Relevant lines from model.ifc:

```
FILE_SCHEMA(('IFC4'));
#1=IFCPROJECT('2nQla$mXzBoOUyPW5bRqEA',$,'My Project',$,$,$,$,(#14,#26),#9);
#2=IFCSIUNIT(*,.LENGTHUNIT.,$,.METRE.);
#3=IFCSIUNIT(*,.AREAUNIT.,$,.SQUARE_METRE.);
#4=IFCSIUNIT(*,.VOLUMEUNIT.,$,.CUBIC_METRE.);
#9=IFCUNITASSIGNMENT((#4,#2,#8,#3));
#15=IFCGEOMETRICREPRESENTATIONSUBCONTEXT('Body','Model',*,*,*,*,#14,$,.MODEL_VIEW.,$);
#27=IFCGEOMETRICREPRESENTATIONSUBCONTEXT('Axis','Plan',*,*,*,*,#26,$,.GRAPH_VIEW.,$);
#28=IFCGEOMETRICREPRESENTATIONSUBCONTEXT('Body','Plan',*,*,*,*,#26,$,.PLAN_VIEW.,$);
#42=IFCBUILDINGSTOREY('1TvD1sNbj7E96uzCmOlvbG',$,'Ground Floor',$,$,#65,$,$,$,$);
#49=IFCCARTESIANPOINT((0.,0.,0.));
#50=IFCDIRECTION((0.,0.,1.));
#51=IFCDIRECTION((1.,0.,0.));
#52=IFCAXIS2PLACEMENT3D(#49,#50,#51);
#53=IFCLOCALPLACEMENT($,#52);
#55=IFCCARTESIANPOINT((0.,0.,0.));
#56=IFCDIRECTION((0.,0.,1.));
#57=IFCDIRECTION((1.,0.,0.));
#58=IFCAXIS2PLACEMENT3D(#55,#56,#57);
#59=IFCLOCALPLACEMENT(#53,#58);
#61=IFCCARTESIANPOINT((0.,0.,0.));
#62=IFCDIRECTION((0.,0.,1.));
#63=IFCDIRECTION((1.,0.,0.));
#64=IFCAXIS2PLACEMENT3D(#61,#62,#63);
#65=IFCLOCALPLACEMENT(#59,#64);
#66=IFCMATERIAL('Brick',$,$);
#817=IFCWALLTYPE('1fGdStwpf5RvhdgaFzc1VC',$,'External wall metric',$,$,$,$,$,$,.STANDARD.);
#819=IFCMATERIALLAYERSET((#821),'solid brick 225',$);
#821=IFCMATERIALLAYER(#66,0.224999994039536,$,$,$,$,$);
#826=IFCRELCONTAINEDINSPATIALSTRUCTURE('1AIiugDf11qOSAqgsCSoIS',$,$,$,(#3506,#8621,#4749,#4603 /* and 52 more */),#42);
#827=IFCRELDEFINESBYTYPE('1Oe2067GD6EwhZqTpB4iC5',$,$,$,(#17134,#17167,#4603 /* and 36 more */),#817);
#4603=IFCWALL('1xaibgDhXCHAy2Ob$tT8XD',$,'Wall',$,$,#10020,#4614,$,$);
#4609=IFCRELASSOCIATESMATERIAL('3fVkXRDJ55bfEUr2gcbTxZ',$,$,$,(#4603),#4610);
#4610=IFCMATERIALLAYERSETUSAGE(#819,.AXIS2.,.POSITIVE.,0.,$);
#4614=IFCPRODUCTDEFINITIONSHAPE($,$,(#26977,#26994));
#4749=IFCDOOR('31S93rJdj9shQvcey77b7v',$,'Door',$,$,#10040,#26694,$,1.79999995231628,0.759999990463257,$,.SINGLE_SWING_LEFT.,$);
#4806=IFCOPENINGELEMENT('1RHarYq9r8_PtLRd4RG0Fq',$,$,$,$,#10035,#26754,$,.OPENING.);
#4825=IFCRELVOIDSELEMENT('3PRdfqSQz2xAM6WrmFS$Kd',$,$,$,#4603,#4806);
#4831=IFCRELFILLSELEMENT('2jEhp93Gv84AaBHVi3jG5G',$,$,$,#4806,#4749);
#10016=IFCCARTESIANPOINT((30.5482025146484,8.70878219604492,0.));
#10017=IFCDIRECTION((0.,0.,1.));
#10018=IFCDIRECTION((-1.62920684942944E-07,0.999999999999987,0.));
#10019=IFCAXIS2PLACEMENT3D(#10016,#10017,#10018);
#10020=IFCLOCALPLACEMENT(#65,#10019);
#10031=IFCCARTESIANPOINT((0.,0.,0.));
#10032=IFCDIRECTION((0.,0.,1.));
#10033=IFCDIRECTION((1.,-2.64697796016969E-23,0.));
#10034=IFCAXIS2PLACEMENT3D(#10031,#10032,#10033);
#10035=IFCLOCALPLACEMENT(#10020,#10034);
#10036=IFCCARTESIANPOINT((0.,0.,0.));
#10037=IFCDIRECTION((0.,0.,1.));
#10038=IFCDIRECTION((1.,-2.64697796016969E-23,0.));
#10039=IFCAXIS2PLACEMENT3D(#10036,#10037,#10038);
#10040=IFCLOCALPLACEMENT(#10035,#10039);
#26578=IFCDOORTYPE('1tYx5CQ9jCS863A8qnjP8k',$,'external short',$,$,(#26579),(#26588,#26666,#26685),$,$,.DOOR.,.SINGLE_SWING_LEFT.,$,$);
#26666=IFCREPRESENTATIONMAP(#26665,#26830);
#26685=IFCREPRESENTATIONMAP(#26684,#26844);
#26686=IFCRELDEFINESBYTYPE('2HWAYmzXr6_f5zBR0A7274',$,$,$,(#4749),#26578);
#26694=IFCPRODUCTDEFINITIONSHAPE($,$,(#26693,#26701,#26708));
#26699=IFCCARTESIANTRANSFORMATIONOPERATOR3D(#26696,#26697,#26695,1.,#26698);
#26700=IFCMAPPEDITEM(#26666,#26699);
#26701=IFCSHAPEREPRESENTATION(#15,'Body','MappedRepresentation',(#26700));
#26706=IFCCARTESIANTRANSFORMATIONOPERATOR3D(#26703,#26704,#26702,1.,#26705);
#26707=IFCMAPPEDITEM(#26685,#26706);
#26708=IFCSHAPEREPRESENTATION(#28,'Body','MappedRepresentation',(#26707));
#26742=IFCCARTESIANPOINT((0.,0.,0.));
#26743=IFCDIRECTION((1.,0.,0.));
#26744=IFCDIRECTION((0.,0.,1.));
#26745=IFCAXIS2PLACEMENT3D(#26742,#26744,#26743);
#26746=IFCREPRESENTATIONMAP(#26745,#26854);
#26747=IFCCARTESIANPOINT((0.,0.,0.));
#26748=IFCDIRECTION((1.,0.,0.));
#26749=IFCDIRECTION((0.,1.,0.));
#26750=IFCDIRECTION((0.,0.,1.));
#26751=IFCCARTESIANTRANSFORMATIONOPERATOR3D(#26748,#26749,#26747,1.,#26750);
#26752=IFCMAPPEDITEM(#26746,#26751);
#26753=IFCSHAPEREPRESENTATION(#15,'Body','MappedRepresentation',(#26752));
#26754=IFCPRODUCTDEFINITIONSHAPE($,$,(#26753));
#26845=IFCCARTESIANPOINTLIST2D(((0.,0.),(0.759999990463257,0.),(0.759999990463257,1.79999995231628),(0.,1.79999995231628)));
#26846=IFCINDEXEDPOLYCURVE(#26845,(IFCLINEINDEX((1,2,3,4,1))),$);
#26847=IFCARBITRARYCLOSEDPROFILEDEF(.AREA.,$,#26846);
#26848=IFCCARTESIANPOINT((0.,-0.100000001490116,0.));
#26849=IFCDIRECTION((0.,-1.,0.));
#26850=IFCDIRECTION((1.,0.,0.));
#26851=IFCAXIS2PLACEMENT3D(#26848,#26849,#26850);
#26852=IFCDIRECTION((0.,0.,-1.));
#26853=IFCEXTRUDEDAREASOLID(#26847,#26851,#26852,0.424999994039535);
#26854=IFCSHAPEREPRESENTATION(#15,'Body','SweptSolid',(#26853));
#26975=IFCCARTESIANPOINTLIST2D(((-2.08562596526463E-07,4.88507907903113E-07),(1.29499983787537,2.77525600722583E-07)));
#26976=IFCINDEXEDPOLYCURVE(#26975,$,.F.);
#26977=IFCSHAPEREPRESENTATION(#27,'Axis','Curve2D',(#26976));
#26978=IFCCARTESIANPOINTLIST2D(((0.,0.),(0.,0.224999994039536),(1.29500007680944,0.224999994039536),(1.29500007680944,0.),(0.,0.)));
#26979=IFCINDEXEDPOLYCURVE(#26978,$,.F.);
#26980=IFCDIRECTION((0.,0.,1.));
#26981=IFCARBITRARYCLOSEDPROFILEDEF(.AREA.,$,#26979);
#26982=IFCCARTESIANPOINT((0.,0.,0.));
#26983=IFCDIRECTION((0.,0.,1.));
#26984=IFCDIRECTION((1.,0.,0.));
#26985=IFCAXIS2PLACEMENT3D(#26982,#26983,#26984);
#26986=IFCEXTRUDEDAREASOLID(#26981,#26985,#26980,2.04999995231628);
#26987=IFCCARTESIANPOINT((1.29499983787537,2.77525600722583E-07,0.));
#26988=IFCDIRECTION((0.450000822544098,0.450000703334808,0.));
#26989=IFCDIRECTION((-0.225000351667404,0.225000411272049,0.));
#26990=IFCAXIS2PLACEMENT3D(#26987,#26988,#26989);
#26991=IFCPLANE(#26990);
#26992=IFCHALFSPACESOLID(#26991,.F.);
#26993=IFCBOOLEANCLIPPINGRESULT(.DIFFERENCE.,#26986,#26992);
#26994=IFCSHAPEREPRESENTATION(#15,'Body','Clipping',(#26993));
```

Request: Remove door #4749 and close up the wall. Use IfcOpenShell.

```python
import ifcopenshell
import ifcopenshell.api.feature
import ifcopenshell.api.root
import ifcopenshell.geom
import ifcopenshell.util.shape

model = ifcopenshell.open("model.ifc")
settings = ifcopenshell.geom.settings()


def volume(element):
    """Net volume in cubic metres, openings subtracted."""
    shape = ifcopenshell.geom.create_shape(settings, element)
    return ifcopenshell.util.shape.get_volume(shape.geometry)


door = model.by_guid("31S93rJdj9shQvcey77b7v")
opening = door.FillsVoids[0].RelatingOpeningElement
wall = opening.VoidsElements[0].RelatingBuildingElement
before = volume(wall)

ifcopenshell.api.root.remove_product(model, product=door)
ifcopenshell.api.feature.remove_feature(model, feature=opening)

after = volume(wall)

print(f"wall volume {before:.3f} -> {after:.3f} m3")

model.write("model_v2.ifc")
```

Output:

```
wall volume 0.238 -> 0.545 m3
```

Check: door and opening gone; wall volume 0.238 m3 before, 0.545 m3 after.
